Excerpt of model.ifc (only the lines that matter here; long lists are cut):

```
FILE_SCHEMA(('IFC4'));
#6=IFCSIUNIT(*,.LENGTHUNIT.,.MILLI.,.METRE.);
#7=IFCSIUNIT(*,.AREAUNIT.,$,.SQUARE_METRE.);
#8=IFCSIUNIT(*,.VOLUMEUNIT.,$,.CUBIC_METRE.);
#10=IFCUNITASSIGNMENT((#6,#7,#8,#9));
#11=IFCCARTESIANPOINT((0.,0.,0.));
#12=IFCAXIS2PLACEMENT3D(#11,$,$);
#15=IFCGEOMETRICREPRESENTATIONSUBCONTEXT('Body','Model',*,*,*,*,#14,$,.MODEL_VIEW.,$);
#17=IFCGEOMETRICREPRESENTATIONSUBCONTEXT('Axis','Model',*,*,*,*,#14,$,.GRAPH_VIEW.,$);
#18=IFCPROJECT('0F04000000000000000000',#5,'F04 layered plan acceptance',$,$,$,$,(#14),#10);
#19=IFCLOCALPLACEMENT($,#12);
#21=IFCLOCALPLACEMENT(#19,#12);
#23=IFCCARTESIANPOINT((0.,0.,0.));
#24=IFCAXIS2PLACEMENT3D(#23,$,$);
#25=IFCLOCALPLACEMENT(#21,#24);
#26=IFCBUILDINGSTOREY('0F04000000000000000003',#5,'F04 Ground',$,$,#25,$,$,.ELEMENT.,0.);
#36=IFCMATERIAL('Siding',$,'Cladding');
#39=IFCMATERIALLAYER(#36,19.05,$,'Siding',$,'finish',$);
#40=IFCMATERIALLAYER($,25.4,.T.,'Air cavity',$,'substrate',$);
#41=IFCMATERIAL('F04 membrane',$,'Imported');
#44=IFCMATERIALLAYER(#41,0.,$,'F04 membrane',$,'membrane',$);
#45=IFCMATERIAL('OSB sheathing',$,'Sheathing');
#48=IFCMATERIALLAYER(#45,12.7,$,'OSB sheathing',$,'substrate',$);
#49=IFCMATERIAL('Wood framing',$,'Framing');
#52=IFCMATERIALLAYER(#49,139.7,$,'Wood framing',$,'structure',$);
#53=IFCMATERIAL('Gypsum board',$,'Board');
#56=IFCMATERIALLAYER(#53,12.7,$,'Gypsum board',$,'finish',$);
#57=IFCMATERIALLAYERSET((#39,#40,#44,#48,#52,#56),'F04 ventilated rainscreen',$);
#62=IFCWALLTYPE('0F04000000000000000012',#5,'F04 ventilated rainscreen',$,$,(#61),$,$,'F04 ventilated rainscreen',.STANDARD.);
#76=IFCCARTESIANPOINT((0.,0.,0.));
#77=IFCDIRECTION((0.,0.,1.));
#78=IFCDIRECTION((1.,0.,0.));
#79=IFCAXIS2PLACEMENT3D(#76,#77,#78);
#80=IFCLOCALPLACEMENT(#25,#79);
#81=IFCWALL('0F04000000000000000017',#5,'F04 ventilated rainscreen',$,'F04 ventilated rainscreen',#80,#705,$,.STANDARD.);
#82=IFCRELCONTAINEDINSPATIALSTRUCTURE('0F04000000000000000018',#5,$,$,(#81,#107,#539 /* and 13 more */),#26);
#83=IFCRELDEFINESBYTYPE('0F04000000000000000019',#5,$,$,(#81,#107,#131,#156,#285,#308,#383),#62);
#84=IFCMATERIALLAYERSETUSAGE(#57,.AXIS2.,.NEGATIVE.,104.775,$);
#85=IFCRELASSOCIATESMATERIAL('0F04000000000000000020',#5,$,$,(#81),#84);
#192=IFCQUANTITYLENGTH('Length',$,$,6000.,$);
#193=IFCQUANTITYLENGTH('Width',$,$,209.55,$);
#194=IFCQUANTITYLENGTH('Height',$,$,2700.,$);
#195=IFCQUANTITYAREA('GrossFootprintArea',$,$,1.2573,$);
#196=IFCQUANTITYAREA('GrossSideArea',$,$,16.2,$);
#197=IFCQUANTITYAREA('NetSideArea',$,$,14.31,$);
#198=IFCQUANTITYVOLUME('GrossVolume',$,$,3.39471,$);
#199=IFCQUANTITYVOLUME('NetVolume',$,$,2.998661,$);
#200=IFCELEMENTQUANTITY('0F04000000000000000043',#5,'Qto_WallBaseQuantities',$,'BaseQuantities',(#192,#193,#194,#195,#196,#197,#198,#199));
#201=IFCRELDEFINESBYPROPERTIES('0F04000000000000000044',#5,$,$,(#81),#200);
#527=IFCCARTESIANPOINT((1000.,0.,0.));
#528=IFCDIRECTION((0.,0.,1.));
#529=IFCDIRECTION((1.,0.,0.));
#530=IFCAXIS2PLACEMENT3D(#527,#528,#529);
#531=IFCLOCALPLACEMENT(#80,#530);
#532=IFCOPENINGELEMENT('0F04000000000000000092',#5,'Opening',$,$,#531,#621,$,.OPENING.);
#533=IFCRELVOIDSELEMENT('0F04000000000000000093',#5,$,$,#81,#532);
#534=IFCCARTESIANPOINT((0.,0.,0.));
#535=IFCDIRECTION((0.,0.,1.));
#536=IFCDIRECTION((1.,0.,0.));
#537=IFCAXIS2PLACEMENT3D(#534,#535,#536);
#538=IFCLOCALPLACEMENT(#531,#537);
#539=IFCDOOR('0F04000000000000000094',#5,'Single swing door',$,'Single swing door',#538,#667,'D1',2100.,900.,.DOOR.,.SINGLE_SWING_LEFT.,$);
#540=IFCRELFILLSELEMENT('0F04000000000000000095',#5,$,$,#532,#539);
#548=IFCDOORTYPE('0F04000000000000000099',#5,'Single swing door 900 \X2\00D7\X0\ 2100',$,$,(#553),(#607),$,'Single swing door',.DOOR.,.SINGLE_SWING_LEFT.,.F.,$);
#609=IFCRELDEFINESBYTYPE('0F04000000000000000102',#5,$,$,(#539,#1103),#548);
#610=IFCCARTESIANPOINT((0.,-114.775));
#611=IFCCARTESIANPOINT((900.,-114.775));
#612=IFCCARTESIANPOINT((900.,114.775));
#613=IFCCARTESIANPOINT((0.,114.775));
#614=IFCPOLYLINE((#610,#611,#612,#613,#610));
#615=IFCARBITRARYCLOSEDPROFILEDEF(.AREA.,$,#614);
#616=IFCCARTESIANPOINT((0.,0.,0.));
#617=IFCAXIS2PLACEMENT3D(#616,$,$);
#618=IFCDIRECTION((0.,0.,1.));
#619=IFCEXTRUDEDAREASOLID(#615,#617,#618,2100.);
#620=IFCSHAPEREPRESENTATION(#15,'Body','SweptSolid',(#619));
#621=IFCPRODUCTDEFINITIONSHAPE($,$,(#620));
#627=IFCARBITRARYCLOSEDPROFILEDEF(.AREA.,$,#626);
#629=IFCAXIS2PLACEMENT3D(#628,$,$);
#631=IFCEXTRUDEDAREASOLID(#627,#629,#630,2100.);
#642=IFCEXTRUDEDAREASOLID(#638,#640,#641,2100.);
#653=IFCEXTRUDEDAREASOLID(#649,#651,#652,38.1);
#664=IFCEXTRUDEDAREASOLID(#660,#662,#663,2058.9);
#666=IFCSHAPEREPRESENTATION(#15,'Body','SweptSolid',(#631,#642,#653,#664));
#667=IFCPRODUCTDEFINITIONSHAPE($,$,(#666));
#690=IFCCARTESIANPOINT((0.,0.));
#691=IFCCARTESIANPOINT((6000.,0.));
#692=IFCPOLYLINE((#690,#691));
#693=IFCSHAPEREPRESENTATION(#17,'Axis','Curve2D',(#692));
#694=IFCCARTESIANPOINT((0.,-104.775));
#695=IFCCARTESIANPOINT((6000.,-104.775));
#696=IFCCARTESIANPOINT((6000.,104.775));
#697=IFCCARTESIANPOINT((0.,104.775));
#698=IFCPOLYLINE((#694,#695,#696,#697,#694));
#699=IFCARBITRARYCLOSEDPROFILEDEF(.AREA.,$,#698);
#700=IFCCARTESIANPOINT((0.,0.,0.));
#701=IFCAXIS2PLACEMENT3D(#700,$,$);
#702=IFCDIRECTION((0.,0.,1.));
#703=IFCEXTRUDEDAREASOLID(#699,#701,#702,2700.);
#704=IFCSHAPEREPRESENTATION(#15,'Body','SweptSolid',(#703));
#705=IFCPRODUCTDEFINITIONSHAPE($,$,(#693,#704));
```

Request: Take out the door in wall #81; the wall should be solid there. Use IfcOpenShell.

```python
import ifcopenshell
import ifcopenshell.api.feature
import ifcopenshell.api.pset
import ifcopenshell.api.root
import ifcopenshell.geom
import ifcopenshell.util.element
import ifcopenshell.util.shape
import ifcopenshell.util.unit

model = ifcopenshell.open("model.ifc")
area_scale = ifcopenshell.util.unit.calculate_unit_scale(model, "AREAUNIT")
volume_scale = ifcopenshell.util.unit.calculate_unit_scale(model, "VOLUMEUNIT")
settings = ifcopenshell.geom.settings()


def volume(element):
    """Net volume in cubic metres, openings subtracted."""
    shape = ifcopenshell.geom.create_shape(settings, element)
    return ifcopenshell.util.shape.get_volume(shape.geometry)


door = model.by_guid("0F04000000000000000094")
opening = door.FillsVoids[0].RelatingOpeningElement
wall = opening.VoidsElements[0].RelatingBuildingElement
before = volume(wall)

ifcopenshell.api.root.remove_product(model, product=door)
ifcopenshell.api.feature.remove_feature(model, feature=opening)

after = volume(wall)
thickness = 0.2096  # wall thickness in metres

# Update the wall's stored quantities.
qto = model.by_id(ifcopenshell.util.element.get_pset(wall, "Qto_WallBaseQuantities", should_inherit=False)["id"])
ifcopenshell.api.pset.edit_qto(model, qto=qto, properties={
    "NetSideArea": after / thickness / area_scale,
    "NetVolume": after / volume_scale,
})

print(f"wall volume {before:.3f} -> {after:.3f} m3")

model.write("model-out.ifc")
```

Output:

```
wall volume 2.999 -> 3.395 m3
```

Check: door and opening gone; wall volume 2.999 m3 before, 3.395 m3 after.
